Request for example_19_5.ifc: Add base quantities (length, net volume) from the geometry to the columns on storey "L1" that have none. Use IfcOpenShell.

First a look at what the model holds.

```python
import ifcopenshell
import ifcopenshell.util.element
import ifcopenshell.util.unit

model = ifcopenshell.open("example_19_5.ifc")
print(model.schema)
for unit_type in ("LENGTHUNIT", "AREAUNIT", "VOLUMEUNIT"):
    print(unit_type, ifcopenshell.util.unit.calculate_unit_scale(model, unit_type))
storey = next(s for s in model.by_type("IfcBuildingStorey") if s.Name == "L1")
columns = [e for e in ifcopenshell.util.element.get_decomposition(storey) if e.is_a("IfcColumn")]
for e in sorted(columns, key=lambda e: e.id()):
    print(e.id(), e.is_a(), e.Name, list(ifcopenshell.util.element.get_psets(e, qtos_only=True)), sep=" | ")
```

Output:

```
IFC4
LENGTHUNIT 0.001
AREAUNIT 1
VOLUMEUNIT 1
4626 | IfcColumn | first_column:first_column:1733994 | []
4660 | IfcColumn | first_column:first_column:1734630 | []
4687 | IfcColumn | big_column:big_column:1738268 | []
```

```python
import ifcopenshell
import ifcopenshell.api.pset
import ifcopenshell.geom
import ifcopenshell.util.element
import ifcopenshell.util.shape
import ifcopenshell.util.unit

model = ifcopenshell.open("example_19_5.ifc")
unit_scale = ifcopenshell.util.unit.calculate_unit_scale(model)
volume_scale = ifcopenshell.util.unit.calculate_unit_scale(model, "VOLUMEUNIT")
settings = ifcopenshell.geom.settings()

storey = next(s for s in model.by_type("IfcBuildingStorey") if s.Name == "L1")
columns = [e for e in ifcopenshell.util.element.get_decomposition(storey) if e.is_a("IfcColumn")]

for e in sorted(columns, key=lambda e: e.id()):
    if ifcopenshell.util.element.get_psets(e, qtos_only=True, should_inherit=False):
        continue
    # Geometry comes back in metres, in the element's own axes.
    shape = ifcopenshell.geom.create_shape(settings, e)
    values = {
        "Length": ifcopenshell.util.shape.get_z(shape.geometry) / unit_scale,
        "NetVolume": ifcopenshell.util.shape.get_volume(shape.geometry) / volume_scale,
    }
    qto = ifcopenshell.api.pset.add_qto(model, product=e, name="Qto_ColumnBaseQuantities")
    ifcopenshell.api.pset.edit_qto(model, qto=qto, properties=values)
    print(e.id(), {k: round(v, 3) for k, v in values.items()})

model.write("example_19_5_edited.ifc")
```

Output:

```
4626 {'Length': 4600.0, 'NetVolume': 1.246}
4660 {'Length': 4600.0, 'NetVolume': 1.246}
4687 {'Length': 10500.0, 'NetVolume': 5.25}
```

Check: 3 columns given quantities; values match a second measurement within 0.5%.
